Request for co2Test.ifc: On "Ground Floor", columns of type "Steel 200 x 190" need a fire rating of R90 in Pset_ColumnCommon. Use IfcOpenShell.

First a look at what the model holds.

```python
import ifcopenshell
import ifcopenshell.util.element

model = ifcopenshell.open("co2Test.ifc")
print(model.schema)
storey = next(s for s in model.by_type("IfcBuildingStorey") if s.Name == "Ground Floor")
columns = [e for e in ifcopenshell.util.element.get_decomposition(storey) if e.is_a("IfcColumn")]
seen = {}
for e in columns:
    element_type = ifcopenshell.util.element.get_type(e)
    key = (element_type.Name if element_type != e and element_type else None, ifcopenshell.util.element.get_pset(e, "Pset_ColumnCommon", "FireRating"))
    seen[key] = seen.get(key, 0) + 1
for (name, value), count in sorted(seen.items(), key=str):
    print(count, "x", name, "|", value)
```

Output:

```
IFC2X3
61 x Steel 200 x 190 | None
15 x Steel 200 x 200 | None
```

```python
import ifcopenshell
import ifcopenshell.api.pset
import ifcopenshell.util.element

model = ifcopenshell.open("co2Test.ifc")

storey = next(s for s in model.by_type("IfcBuildingStorey") if s.Name == "Ground Floor")
columns = [e for e in ifcopenshell.util.element.get_decomposition(storey) if e.is_a("IfcColumn")]

count = 0
for e in columns:
    element_type = ifcopenshell.util.element.get_type(e)
    if element_type in (None, e) or element_type.Name != "Steel 200 x 190":
        continue
    # add_pset returns the element's existing set when there is one.
    pset = ifcopenshell.api.pset.add_pset(model, product=e, name="Pset_ColumnCommon")
    ifcopenshell.api.pset.edit_pset(model, pset=pset, properties={"FireRating": "R90"})
    count += 1

print(count, "columns updated")

model.write("co2Test_v2.ifc")
```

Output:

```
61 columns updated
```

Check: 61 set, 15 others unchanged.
